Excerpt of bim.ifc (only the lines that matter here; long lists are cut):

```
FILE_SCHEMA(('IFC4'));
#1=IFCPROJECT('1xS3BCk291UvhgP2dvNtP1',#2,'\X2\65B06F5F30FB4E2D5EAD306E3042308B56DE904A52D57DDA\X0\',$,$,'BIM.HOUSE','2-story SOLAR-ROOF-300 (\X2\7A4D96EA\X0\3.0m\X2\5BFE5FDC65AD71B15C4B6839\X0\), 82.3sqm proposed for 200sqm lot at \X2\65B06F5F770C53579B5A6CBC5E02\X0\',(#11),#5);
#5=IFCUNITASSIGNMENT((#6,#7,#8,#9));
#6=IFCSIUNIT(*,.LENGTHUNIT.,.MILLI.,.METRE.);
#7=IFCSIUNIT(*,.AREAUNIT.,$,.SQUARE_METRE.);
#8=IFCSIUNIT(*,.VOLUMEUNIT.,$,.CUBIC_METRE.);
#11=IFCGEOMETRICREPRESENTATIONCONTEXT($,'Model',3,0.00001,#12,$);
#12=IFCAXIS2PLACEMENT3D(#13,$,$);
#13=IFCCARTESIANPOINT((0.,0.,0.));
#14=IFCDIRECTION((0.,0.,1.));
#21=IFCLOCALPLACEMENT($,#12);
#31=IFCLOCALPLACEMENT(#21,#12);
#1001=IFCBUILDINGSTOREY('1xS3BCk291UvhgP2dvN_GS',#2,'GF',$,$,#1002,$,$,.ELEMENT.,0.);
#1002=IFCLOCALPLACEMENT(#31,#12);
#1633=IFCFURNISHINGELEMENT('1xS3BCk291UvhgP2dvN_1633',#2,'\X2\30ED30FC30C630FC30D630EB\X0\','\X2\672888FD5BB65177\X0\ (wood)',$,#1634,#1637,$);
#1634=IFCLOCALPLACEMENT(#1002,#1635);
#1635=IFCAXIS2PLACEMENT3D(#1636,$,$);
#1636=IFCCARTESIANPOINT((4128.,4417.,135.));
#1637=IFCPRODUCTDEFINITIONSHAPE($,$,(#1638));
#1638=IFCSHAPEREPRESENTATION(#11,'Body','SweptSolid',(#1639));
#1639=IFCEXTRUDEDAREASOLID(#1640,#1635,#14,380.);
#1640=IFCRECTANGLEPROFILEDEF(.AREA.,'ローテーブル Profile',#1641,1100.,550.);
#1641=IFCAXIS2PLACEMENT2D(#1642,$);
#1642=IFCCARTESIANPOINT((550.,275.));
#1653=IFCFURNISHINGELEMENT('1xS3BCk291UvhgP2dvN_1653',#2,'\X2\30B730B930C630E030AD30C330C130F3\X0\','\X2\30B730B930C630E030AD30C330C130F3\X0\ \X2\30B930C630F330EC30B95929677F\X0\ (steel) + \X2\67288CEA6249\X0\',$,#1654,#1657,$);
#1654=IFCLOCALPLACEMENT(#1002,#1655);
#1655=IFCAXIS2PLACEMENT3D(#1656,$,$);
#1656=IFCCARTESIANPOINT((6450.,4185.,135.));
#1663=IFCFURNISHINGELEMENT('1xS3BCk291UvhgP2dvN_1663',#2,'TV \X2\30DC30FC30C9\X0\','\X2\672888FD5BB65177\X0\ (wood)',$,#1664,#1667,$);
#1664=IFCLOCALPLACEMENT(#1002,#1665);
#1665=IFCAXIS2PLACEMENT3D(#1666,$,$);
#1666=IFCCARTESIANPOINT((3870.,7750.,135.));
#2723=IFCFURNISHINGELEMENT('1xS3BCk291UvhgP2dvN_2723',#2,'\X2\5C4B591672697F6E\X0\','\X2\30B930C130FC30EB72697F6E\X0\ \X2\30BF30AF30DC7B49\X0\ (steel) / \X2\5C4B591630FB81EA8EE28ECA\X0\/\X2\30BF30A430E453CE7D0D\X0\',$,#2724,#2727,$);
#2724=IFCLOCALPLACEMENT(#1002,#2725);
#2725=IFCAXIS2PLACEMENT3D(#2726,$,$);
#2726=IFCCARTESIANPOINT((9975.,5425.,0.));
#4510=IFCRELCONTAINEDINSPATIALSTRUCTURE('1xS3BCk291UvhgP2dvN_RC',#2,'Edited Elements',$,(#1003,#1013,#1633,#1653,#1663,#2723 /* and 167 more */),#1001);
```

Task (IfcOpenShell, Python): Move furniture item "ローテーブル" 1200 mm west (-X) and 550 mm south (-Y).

```python
import ifcopenshell
import ifcopenshell.api.geometry
import ifcopenshell.util.placement
import ifcopenshell.util.unit

model = ifcopenshell.open("bim.ifc")
unit_scale = ifcopenshell.util.unit.calculate_unit_scale(model)

item = model.by_guid("1xS3BCk291UvhgP2dvN_1633")
matrix = ifcopenshell.util.placement.get_local_placement(item.ObjectPlacement)
matrix[0, 3] -= 1.2 / unit_scale
matrix[1, 3] -= 0.55 / unit_scale
ifcopenshell.api.geometry.edit_object_placement(model, product=item, matrix=matrix, is_si=False)

print(ifcopenshell.util.placement.get_local_placement(item.ObjectPlacement).round(3) + 0.0)

model.write("bim_v2.ifc")
```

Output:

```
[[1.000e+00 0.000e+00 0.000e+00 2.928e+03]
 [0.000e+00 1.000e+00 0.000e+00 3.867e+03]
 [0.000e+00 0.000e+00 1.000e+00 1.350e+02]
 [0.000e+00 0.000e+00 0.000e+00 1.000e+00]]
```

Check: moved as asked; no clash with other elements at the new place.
